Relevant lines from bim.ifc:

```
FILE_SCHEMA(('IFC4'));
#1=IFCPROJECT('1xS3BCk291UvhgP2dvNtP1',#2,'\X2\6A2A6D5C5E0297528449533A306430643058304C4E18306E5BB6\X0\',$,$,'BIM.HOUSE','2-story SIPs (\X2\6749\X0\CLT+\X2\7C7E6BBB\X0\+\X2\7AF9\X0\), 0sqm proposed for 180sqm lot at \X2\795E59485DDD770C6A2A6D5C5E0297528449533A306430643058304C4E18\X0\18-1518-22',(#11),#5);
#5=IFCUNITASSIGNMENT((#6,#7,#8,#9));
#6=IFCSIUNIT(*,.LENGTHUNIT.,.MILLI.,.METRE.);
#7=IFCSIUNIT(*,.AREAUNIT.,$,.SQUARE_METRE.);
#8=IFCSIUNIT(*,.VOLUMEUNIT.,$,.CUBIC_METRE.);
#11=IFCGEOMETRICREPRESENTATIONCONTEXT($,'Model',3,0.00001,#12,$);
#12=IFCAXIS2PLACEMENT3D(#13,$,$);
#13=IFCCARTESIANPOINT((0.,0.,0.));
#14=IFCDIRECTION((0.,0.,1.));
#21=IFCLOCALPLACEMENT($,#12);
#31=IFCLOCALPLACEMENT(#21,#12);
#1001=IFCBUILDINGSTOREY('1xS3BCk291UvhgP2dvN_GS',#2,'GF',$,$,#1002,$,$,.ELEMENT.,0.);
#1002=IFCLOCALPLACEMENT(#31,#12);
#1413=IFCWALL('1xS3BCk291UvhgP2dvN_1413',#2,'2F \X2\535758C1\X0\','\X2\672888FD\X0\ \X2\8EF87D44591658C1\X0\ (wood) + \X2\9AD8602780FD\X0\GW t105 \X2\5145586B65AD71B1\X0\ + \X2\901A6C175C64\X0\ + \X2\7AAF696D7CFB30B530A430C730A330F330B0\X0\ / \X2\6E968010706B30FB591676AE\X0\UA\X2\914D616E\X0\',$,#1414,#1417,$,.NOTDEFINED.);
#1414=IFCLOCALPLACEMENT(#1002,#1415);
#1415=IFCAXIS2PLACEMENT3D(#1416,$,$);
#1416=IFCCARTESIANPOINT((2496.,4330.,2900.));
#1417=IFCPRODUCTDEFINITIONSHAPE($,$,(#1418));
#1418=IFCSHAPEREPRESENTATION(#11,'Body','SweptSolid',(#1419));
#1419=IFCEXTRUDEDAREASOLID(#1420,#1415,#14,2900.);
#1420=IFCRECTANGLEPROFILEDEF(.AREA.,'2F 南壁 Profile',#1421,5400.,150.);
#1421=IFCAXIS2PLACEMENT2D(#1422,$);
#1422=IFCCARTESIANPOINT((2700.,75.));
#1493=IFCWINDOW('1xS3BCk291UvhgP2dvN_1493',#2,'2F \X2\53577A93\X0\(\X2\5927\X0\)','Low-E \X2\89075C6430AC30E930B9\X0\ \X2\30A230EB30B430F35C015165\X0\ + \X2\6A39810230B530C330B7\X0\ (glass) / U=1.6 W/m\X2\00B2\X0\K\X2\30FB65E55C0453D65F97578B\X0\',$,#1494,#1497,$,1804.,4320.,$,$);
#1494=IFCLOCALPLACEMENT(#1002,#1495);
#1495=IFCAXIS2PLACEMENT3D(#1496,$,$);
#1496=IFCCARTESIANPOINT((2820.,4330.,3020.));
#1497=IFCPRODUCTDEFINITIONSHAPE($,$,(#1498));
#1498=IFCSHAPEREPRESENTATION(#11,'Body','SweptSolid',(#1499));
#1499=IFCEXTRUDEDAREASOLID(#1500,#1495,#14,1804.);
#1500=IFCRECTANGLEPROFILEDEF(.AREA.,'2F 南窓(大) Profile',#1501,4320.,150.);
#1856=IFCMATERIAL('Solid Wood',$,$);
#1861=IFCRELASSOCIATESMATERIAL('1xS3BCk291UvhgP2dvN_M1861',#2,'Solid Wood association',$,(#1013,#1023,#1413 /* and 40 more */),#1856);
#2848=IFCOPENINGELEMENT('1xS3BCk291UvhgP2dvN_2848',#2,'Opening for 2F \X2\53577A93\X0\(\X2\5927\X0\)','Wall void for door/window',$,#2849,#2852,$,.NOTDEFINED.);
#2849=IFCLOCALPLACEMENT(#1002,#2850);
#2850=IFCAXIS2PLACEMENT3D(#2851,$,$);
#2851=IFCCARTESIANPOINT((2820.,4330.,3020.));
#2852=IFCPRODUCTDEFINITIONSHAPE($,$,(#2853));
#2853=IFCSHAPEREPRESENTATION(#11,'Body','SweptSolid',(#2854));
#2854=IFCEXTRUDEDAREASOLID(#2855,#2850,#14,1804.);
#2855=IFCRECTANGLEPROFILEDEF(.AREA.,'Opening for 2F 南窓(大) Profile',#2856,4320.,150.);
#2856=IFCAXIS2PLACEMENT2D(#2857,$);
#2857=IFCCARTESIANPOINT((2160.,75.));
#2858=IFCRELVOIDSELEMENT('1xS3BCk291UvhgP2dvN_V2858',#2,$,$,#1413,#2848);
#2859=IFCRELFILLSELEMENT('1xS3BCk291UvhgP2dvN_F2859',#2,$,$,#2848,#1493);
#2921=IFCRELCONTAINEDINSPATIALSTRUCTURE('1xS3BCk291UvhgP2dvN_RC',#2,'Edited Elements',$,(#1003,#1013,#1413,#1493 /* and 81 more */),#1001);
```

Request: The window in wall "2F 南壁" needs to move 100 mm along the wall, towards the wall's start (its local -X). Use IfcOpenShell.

```python
import ifcopenshell
import ifcopenshell.api.geometry
import ifcopenshell.util.placement
import ifcopenshell.util.unit

model = ifcopenshell.open("bim.ifc")
unit_scale = ifcopenshell.util.unit.calculate_unit_scale(model)

window = model.by_guid("1xS3BCk291UvhgP2dvN_1493")
opening = window.FillsVoids[0].RelatingOpeningElement
wall = opening.VoidsElements[0].RelatingBuildingElement

wall_matrix = ifcopenshell.util.placement.get_local_placement(wall.ObjectPlacement)
shift = wall_matrix[:3, 0] * -0.1 / unit_scale
before = ifcopenshell.util.placement.get_local_placement(window.ObjectPlacement)[:3, 3].copy()

# The window is not placed relative to its opening, so move both.
for product in (opening, window):
    matrix = ifcopenshell.util.placement.get_local_placement(product.ObjectPlacement)
    matrix[:3, 3] += shift
    ifcopenshell.api.geometry.edit_object_placement(model, product=product, matrix=matrix, is_si=False)

after = ifcopenshell.util.placement.get_local_placement(window.ObjectPlacement)[:3, 3]
print("window moved by", (after - before).round(3) + 0.0)

model.write("bim_edited.ifc")
```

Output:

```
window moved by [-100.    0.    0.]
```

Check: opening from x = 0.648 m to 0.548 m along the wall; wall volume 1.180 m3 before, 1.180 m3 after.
